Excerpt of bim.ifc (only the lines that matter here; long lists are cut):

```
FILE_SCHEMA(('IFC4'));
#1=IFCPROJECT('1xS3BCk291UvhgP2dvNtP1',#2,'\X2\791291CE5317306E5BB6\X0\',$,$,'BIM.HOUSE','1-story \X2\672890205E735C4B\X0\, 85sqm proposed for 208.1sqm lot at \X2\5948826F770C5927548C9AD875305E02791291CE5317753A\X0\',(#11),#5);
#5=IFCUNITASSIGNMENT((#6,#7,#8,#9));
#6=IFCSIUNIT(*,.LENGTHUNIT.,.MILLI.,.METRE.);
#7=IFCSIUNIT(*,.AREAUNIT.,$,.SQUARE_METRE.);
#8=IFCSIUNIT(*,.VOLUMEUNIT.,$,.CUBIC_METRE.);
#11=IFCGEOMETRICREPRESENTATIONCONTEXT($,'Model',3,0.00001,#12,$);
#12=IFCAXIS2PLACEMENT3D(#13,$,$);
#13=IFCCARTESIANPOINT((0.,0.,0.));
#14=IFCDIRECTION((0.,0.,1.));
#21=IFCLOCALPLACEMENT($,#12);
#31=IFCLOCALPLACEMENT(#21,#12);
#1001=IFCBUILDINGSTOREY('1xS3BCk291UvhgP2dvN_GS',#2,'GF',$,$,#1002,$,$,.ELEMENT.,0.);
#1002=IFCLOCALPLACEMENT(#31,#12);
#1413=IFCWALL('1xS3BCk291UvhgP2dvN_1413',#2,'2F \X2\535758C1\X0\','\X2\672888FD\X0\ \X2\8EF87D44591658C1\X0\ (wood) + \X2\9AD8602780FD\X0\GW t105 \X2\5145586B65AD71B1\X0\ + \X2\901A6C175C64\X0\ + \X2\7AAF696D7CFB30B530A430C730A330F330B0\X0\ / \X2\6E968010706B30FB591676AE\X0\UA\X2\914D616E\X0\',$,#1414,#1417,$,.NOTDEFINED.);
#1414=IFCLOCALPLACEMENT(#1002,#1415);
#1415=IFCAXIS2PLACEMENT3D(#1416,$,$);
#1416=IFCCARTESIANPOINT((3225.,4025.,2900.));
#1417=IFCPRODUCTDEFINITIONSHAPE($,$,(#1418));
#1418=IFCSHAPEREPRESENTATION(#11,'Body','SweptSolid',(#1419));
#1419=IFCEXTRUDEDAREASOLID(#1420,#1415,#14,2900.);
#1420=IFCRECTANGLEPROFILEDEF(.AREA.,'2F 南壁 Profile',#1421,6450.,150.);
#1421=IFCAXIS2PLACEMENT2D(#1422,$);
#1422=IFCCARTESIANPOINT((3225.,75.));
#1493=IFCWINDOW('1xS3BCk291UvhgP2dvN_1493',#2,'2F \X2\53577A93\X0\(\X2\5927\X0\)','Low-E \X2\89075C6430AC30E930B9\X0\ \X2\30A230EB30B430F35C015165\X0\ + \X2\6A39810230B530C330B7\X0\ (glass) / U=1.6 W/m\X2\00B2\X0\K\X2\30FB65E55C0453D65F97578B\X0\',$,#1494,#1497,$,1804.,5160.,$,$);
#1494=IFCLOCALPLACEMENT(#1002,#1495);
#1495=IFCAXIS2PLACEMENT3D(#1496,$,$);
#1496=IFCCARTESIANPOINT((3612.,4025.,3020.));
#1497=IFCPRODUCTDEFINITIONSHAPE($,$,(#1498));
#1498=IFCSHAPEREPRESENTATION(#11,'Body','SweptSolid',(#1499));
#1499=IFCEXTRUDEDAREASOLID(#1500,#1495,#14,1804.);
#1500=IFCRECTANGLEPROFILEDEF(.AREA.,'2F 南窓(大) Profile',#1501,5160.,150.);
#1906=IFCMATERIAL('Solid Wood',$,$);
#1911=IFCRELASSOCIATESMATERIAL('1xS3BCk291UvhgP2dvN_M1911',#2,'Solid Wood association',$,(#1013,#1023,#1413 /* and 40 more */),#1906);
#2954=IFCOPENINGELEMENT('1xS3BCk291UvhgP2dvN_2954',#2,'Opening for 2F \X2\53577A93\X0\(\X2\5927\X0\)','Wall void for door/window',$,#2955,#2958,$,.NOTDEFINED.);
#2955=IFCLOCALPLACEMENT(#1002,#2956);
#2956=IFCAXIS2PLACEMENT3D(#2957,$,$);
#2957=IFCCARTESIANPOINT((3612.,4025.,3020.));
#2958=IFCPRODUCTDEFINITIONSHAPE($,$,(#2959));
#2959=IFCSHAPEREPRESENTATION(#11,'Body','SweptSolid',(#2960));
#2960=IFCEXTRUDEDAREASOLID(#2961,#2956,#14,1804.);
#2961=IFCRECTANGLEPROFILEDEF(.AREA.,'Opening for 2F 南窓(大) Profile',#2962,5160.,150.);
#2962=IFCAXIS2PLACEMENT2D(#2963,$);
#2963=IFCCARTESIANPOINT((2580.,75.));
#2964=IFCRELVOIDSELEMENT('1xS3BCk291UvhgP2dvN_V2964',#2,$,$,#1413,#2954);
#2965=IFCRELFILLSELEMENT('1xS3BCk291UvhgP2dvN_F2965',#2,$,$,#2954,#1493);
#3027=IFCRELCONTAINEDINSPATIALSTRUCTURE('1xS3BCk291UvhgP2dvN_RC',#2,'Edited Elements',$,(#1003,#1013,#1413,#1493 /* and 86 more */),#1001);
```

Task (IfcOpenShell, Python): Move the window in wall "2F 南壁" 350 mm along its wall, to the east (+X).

```python
import ifcopenshell
import ifcopenshell.api.geometry
import ifcopenshell.util.placement
import ifcopenshell.util.unit

model = ifcopenshell.open("bim.ifc")
unit_scale = ifcopenshell.util.unit.calculate_unit_scale(model)

window = model.by_guid("1xS3BCk291UvhgP2dvN_1493")
opening = window.FillsVoids[0].RelatingOpeningElement
wall = opening.VoidsElements[0].RelatingBuildingElement

wall_matrix = ifcopenshell.util.placement.get_local_placement(wall.ObjectPlacement)
shift = wall_matrix[:3, 0] * 0.35 / unit_scale
before = ifcopenshell.util.placement.get_local_placement(window.ObjectPlacement)[:3, 3].copy()

# The window is not placed relative to its opening, so move both.
for product in (opening, window):
    matrix = ifcopenshell.util.placement.get_local_placement(product.ObjectPlacement)
    matrix[:3, 3] += shift
    ifcopenshell.api.geometry.edit_object_placement(model, product=product, matrix=matrix, is_si=False)

after = ifcopenshell.util.placement.get_local_placement(window.ObjectPlacement)[:3, 3]
print("window moved by", (after - before).round(3) + 0.0)

model.write("bim_rev.ifc")
```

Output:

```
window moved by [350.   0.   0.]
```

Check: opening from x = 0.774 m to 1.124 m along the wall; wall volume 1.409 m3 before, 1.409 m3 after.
